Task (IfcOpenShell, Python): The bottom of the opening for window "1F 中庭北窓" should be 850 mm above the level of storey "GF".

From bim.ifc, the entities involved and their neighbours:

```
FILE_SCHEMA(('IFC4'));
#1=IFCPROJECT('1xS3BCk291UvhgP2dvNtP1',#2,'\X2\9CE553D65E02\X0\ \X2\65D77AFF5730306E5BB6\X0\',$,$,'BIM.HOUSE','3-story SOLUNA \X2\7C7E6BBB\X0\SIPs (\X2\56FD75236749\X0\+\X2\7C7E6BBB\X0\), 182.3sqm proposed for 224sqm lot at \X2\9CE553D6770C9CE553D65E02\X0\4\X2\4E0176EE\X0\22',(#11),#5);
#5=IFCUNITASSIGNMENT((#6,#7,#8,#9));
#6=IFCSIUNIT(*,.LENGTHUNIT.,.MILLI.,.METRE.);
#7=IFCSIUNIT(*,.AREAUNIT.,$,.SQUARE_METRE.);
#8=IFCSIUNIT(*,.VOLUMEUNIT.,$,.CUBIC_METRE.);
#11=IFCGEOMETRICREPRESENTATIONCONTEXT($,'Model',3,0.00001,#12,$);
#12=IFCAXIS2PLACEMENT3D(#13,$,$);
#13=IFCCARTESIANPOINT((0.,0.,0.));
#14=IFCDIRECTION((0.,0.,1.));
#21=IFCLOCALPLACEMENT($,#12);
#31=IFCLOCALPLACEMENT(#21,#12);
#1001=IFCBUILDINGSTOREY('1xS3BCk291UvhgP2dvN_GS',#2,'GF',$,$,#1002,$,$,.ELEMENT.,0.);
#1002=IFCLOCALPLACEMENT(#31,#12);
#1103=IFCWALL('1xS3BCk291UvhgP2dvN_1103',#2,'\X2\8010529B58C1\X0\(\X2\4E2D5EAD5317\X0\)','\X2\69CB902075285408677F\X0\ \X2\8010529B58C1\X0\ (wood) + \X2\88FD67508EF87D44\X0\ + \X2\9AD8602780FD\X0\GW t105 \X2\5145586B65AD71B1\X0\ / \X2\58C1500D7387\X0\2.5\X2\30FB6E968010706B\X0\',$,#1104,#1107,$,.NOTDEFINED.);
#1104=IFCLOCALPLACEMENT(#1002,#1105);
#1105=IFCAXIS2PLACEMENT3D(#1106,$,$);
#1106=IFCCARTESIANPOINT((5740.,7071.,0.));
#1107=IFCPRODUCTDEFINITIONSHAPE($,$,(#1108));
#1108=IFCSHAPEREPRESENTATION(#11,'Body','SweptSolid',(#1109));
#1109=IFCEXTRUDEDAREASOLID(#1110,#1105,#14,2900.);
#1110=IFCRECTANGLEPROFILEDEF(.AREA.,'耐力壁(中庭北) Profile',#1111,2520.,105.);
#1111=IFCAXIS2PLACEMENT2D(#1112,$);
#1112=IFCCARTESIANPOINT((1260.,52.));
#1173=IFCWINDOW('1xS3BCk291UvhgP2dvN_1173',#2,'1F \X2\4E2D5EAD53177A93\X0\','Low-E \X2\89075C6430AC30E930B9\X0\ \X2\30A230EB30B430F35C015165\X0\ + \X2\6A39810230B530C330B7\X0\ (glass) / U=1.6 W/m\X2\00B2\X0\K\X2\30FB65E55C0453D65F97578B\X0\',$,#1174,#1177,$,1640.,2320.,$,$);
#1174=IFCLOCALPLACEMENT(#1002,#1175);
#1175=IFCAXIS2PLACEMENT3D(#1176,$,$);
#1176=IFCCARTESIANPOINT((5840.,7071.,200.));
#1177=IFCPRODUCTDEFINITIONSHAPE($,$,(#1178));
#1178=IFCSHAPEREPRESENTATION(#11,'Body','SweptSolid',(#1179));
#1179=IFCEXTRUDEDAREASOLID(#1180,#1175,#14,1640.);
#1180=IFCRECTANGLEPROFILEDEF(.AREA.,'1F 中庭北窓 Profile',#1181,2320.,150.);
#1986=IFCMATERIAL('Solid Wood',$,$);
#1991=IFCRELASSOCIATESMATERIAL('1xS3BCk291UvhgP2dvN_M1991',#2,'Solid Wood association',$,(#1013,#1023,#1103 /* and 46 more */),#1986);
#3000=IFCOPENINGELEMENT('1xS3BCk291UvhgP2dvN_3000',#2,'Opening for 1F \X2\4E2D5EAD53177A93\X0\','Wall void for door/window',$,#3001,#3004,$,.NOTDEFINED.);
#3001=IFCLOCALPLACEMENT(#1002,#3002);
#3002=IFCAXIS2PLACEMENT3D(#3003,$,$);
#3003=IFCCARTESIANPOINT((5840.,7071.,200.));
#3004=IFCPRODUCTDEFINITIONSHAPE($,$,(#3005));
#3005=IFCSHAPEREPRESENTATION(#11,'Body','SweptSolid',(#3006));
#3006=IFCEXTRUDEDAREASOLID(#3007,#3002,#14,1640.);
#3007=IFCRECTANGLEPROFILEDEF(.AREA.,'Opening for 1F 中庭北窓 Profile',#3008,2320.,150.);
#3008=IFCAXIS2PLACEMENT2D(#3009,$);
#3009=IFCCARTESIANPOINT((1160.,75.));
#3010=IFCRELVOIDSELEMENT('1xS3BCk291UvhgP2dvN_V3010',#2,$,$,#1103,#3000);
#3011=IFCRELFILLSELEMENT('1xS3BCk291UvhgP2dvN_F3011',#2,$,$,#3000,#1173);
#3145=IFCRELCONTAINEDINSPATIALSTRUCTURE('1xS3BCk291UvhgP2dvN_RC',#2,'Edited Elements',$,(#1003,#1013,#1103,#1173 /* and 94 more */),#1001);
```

```python
import numpy as np
import ifcopenshell
import ifcopenshell.api.geometry
import ifcopenshell.geom
import ifcopenshell.util.element
import ifcopenshell.util.placement
import ifcopenshell.util.shape
import ifcopenshell.util.unit

model = ifcopenshell.open("bim.ifc")
unit_scale = ifcopenshell.util.unit.calculate_unit_scale(model)

window = model.by_id(1173)
opening = window.FillsVoids[0].RelatingOpeningElement
storey = ifcopenshell.util.element.get_container(window, ifc_class="IfcBuildingStorey")
level = ifcopenshell.util.placement.get_local_placement(storey.ObjectPlacement)[2, 3]

# The opening's origin need not be at the sill, so measure its lowest point.
shape = ifcopenshell.geom.create_shape(ifcopenshell.geom.settings(), opening)
bottom = ifcopenshell.util.shape.get_shape_bottom_elevation(shape, shape.geometry) / unit_scale
dz = level + 0.85 / unit_scale - bottom

shift = np.array([0.0, 0.0, dz])
# The window is not placed relative to its opening, so move both.
for product in (opening, window):
    matrix = ifcopenshell.util.placement.get_local_placement(product.ObjectPlacement)
    matrix[:3, 3] += shift
    ifcopenshell.api.geometry.edit_object_placement(model, product=product, matrix=matrix, is_si=False)

print(f"moved by {dz * unit_scale:+.3f} m")

model.write("bim-out.ifc")
```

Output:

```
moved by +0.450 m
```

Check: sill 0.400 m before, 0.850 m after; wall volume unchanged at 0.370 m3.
